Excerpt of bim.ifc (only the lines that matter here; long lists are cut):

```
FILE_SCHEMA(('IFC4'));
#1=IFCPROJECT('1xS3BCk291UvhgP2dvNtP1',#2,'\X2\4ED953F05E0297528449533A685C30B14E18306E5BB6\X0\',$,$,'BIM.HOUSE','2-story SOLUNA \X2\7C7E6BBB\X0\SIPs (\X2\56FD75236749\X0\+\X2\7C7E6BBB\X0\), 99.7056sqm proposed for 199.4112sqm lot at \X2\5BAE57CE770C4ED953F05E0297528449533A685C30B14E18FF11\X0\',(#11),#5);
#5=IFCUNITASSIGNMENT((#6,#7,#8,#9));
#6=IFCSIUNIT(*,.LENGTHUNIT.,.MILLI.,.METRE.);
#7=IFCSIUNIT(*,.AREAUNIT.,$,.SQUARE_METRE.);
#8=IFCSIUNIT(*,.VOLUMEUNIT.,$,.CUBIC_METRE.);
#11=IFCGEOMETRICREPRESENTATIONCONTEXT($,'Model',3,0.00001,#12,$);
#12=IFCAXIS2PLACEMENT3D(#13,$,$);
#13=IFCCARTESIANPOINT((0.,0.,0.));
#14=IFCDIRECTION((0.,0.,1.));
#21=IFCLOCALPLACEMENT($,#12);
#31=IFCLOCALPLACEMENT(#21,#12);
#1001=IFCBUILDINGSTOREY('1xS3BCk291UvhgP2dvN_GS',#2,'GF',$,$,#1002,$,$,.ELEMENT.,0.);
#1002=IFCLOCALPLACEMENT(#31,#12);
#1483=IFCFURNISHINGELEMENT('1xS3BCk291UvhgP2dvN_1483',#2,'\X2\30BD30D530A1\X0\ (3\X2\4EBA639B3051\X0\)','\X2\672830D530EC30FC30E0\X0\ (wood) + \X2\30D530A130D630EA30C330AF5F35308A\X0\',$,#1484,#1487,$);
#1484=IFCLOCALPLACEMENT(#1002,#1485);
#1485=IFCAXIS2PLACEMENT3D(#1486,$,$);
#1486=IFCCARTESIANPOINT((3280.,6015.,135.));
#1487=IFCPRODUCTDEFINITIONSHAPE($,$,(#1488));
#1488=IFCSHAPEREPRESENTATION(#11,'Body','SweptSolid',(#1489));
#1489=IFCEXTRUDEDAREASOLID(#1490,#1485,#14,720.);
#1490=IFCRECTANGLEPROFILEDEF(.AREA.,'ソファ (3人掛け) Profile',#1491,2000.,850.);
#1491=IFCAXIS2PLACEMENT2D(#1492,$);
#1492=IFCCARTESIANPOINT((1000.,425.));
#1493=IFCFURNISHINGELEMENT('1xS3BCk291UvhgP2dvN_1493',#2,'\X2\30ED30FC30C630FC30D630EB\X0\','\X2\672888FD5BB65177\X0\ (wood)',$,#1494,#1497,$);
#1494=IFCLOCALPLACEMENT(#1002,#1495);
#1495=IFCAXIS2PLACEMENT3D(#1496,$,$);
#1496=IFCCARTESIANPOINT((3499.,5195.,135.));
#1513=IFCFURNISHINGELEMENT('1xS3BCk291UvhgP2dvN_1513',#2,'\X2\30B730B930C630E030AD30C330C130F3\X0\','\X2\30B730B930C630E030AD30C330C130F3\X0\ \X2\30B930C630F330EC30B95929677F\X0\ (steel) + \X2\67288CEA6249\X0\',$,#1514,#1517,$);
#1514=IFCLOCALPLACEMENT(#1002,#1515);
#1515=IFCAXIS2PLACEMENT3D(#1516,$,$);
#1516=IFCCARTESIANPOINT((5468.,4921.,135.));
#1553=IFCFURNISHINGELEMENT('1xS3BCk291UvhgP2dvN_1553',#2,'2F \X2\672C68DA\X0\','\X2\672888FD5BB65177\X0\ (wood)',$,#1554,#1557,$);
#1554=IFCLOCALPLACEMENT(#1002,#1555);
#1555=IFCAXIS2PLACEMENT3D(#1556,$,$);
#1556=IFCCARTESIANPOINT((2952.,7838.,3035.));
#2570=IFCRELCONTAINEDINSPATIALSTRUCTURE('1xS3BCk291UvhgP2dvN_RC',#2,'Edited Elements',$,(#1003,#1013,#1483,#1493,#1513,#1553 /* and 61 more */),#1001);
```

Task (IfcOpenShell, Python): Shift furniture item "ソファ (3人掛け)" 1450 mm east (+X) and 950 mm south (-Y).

```python
import ifcopenshell
import ifcopenshell.api.geometry
import ifcopenshell.util.placement
import ifcopenshell.util.unit

model = ifcopenshell.open("bim.ifc")
unit_scale = ifcopenshell.util.unit.calculate_unit_scale(model)

item = model.by_guid("1xS3BCk291UvhgP2dvN_1483")
matrix = ifcopenshell.util.placement.get_local_placement(item.ObjectPlacement)
matrix[0, 3] += 1.45 / unit_scale
matrix[1, 3] -= 0.95 / unit_scale
ifcopenshell.api.geometry.edit_object_placement(model, product=item, matrix=matrix, is_si=False)

print(ifcopenshell.util.placement.get_local_placement(item.ObjectPlacement).round(3) + 0.0)

model.write("bim_updated.ifc")
```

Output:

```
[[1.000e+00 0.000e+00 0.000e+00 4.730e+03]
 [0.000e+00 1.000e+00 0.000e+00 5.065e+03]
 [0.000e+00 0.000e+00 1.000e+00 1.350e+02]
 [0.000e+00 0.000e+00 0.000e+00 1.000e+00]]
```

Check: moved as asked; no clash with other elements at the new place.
